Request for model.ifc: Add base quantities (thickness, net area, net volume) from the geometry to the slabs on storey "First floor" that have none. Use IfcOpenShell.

First a look at what the model holds.

```python
import ifcopenshell
import ifcopenshell.util.element
import ifcopenshell.util.unit

model = ifcopenshell.open("model.ifc")
print(model.schema)
for unit_type in ("LENGTHUNIT", "AREAUNIT", "VOLUMEUNIT"):
    print(unit_type, ifcopenshell.util.unit.calculate_unit_scale(model, unit_type))
storey = next(s for s in model.by_type("IfcBuildingStorey") if s.Name == "First floor")
slabs = [e for e in ifcopenshell.util.element.get_decomposition(storey) if e.is_a("IfcSlab")]
for e in sorted(slabs, key=lambda e: e.id()):
    print(e.id(), e.is_a(), e.Name, list(ifcopenshell.util.element.get_psets(e, qtos_only=True)), sep=" | ")
```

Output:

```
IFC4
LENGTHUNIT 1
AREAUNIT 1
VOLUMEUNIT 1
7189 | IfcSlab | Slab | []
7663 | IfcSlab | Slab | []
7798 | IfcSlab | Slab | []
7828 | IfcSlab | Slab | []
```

```python
import ifcopenshell
import ifcopenshell.api.pset
import ifcopenshell.geom
import ifcopenshell.util.element
import ifcopenshell.util.shape
import ifcopenshell.util.unit

model = ifcopenshell.open("model.ifc")
unit_scale = ifcopenshell.util.unit.calculate_unit_scale(model)
area_scale = ifcopenshell.util.unit.calculate_unit_scale(model, "AREAUNIT")
volume_scale = ifcopenshell.util.unit.calculate_unit_scale(model, "VOLUMEUNIT")
settings = ifcopenshell.geom.settings()

storey = next(s for s in model.by_type("IfcBuildingStorey") if s.Name == "First floor")
slabs = [e for e in ifcopenshell.util.element.get_decomposition(storey) if e.is_a("IfcSlab")]

for e in sorted(slabs, key=lambda e: e.id()):
    if ifcopenshell.util.element.get_psets(e, qtos_only=True, should_inherit=False):
        continue
    # Geometry comes back in metres, in the element's own axes.
    shape = ifcopenshell.geom.create_shape(settings, e)
    values = {
        "Width": ifcopenshell.util.shape.get_z(shape.geometry) / unit_scale,
        "NetArea": ifcopenshell.util.shape.get_footprint_area(shape.geometry) / area_scale,
        "NetVolume": ifcopenshell.util.shape.get_volume(shape.geometry) / volume_scale,
    }
    qto = ifcopenshell.api.pset.add_qto(model, product=e, name="Qto_SlabBaseQuantities")
    ifcopenshell.api.pset.edit_qto(model, qto=qto, properties=values)
    print(e.id(), {k: round(v, 3) for k, v in values.items()})

model.write("model-out.ifc")
```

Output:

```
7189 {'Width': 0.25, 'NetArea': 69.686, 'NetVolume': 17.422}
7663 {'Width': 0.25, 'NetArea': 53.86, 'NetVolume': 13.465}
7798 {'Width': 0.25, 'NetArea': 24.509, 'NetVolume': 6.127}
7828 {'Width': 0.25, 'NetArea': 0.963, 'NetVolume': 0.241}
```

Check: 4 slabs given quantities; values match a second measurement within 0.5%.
